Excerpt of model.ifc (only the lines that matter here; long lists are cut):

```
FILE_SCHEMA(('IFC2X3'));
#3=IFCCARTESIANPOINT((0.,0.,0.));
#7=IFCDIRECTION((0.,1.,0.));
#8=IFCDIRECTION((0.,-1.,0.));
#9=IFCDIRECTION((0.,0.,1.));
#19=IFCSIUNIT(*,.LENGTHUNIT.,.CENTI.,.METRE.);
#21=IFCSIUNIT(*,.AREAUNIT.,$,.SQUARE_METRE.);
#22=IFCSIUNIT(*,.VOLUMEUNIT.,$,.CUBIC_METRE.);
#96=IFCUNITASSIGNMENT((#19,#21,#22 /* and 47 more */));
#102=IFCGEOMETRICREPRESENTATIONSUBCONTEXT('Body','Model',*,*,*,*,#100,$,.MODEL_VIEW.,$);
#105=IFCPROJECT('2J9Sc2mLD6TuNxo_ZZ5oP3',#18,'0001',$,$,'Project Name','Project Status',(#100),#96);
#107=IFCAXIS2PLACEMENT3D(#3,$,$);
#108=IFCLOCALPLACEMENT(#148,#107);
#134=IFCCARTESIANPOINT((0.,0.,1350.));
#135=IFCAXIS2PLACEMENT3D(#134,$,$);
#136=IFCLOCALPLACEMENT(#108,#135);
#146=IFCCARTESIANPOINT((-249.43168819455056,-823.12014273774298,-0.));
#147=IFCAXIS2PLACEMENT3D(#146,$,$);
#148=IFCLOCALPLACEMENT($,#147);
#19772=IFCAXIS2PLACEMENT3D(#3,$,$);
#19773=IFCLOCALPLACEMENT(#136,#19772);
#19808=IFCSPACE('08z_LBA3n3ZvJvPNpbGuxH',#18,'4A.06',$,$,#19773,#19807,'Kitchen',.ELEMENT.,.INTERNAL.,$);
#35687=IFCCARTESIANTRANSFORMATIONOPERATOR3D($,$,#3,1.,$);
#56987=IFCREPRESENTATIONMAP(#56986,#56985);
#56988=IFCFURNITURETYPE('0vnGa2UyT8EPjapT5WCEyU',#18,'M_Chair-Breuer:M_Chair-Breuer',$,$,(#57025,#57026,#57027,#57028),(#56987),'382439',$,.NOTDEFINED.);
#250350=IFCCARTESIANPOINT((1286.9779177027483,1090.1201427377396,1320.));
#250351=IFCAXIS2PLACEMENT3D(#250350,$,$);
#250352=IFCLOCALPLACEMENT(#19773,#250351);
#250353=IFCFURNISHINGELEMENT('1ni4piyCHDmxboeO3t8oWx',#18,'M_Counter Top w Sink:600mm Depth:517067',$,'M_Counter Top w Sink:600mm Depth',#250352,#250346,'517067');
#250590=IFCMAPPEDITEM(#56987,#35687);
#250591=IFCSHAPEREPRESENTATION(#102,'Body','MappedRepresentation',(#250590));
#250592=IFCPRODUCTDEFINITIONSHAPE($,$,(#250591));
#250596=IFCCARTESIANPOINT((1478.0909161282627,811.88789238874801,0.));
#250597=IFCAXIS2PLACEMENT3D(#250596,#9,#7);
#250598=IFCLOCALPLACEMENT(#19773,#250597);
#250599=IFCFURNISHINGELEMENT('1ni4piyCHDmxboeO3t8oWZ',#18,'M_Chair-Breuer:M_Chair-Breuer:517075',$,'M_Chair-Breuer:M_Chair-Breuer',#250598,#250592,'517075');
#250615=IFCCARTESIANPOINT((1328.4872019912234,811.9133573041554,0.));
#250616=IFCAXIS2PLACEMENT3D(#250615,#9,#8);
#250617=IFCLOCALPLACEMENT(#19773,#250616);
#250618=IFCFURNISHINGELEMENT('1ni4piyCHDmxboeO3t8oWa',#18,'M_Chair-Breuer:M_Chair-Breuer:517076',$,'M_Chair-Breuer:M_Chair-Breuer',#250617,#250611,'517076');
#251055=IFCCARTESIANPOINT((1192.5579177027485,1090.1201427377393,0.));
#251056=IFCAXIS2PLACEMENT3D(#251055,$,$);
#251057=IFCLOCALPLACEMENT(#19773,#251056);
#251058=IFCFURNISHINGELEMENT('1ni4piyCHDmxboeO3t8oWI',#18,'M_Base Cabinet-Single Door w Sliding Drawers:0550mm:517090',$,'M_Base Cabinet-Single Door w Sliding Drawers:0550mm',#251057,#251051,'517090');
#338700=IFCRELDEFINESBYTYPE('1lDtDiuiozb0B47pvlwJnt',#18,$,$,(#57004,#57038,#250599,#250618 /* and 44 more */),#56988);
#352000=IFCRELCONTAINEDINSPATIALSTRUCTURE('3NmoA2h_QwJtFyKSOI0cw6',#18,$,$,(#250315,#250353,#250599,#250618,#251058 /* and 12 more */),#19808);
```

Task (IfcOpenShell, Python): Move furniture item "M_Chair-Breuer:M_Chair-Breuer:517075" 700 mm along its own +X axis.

```python
import ifcopenshell
import ifcopenshell.api.geometry
import ifcopenshell.util.placement
import ifcopenshell.util.unit

model = ifcopenshell.open("model.ifc")
unit_scale = ifcopenshell.util.unit.calculate_unit_scale(model)

item = model.by_guid("1ni4piyCHDmxboeO3t8oWZ")
matrix = ifcopenshell.util.placement.get_local_placement(item.ObjectPlacement)
matrix[:3, 3] += matrix[:3, 0] * 0.7 / unit_scale
ifcopenshell.api.geometry.edit_object_placement(model, product=item, matrix=matrix, is_si=False)

print(ifcopenshell.util.placement.get_local_placement(item.ObjectPlacement).round(3) + 0.0)

model.write("model_updated.ifc")
```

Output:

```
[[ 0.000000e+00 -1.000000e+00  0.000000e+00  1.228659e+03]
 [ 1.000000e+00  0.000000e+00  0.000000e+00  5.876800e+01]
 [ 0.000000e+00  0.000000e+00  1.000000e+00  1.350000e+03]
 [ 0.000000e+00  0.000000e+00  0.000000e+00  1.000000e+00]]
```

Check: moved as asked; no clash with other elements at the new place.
